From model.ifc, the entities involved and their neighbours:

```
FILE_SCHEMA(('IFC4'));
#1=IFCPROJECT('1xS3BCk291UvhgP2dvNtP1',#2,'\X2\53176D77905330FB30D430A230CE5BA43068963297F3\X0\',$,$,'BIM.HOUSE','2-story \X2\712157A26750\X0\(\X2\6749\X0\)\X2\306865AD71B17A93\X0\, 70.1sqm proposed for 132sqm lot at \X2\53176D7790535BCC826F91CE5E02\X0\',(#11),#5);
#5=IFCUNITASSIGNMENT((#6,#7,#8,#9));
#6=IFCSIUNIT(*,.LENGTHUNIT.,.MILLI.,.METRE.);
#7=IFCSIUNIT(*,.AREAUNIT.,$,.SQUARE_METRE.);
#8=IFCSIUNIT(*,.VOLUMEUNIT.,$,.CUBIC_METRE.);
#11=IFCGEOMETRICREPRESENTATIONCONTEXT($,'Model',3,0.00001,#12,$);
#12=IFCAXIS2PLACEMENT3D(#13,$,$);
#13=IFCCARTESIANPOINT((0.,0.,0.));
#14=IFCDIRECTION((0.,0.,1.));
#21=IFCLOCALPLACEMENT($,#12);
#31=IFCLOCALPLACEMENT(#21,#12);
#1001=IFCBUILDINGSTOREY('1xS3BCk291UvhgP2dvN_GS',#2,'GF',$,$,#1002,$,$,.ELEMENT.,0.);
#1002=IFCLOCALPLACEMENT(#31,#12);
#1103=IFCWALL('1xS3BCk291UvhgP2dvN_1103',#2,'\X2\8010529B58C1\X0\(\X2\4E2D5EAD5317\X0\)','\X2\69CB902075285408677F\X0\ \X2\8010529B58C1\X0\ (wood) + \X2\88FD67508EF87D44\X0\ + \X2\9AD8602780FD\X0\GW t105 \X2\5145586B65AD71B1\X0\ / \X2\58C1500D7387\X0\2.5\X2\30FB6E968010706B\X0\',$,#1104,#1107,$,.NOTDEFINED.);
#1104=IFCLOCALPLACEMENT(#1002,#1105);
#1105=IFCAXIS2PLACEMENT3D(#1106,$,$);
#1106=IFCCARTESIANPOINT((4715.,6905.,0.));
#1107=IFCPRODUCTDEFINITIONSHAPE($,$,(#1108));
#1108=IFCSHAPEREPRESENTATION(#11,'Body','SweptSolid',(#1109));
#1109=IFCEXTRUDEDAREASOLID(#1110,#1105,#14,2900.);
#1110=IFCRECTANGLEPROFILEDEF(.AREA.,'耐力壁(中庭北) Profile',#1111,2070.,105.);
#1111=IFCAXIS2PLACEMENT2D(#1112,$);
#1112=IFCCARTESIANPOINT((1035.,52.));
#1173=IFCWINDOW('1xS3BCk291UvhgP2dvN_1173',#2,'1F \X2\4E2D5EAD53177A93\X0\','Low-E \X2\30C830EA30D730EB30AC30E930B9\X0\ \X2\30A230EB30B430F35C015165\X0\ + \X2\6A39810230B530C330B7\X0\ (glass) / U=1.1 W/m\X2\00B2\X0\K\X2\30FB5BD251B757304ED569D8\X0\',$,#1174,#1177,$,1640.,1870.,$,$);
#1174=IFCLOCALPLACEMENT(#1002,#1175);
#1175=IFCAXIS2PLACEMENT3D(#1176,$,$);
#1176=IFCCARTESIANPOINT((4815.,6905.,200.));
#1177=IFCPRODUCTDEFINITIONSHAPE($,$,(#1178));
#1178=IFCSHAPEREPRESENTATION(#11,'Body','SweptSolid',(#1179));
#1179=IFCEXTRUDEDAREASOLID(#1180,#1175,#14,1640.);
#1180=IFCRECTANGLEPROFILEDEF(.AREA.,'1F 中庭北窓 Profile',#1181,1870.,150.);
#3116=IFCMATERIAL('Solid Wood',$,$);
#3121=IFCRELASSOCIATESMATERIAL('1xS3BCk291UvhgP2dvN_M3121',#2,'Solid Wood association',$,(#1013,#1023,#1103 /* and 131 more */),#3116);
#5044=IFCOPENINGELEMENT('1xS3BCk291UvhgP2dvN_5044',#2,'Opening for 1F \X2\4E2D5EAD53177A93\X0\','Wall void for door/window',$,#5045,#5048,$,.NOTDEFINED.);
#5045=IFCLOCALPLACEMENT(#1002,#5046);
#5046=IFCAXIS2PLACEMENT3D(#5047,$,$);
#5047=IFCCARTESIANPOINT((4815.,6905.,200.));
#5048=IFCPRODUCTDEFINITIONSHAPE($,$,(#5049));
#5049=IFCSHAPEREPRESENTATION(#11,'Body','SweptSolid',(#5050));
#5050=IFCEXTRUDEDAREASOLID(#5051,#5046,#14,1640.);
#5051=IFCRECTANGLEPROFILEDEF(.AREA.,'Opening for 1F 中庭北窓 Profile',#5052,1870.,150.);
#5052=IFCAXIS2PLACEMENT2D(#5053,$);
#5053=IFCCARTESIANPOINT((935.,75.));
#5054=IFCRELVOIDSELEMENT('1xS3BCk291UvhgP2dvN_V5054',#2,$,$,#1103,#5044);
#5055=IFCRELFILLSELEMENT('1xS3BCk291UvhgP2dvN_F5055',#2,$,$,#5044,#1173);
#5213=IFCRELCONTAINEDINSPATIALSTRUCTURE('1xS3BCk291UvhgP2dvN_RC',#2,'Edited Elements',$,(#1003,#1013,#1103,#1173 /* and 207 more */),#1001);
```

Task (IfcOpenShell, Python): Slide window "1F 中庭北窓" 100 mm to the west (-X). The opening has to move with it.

```python
import ifcopenshell
import ifcopenshell.api.geometry
import ifcopenshell.util.placement
import ifcopenshell.util.unit

model = ifcopenshell.open("model.ifc")
unit_scale = ifcopenshell.util.unit.calculate_unit_scale(model)

window = model.by_guid("1xS3BCk291UvhgP2dvN_1173")
opening = window.FillsVoids[0].RelatingOpeningElement
wall = opening.VoidsElements[0].RelatingBuildingElement

wall_matrix = ifcopenshell.util.placement.get_local_placement(wall.ObjectPlacement)
shift = wall_matrix[:3, 0] * -0.1 / unit_scale
before = ifcopenshell.util.placement.get_local_placement(window.ObjectPlacement)[:3, 3].copy()

# The window is not placed relative to its opening, so move both.
for product in (opening, window):
    matrix = ifcopenshell.util.placement.get_local_placement(product.ObjectPlacement)
    matrix[:3, 3] += shift
    ifcopenshell.api.geometry.edit_object_placement(model, product=product, matrix=matrix, is_si=False)

after = ifcopenshell.util.placement.get_local_placement(window.ObjectPlacement)[:3, 3]
print("window moved by", (after - before).round(3) + 0.0)

model.write("model-out.ifc")
```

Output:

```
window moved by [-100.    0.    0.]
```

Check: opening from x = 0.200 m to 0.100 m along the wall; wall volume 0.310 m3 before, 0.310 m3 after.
